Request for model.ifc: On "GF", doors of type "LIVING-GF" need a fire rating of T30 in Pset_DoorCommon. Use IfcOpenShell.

First a look at what the model holds.

```python
import ifcopenshell
import ifcopenshell.util.element

model = ifcopenshell.open("model.ifc")
print(model.schema)
storey = next(s for s in model.by_type("IfcBuildingStorey") if s.Name == "GF")
doors = [e for e in ifcopenshell.util.element.get_decomposition(storey) if e.is_a("IfcDoor")]
seen = {}
for e in doors:
    element_type = ifcopenshell.util.element.get_type(e)
    key = (element_type.Name if element_type != e and element_type else None, ifcopenshell.util.element.get_pset(e, "Pset_DoorCommon", "FireRating"))
    seen[key] = seen.get(key, 0) + 1
for (name, value), count in sorted(seen.items(), key=str):
    print(count, "x", name, "|", value)
```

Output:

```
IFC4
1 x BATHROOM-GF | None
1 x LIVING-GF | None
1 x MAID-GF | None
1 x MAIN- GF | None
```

```python
import ifcopenshell
import ifcopenshell.api.pset
import ifcopenshell.util.element

model = ifcopenshell.open("model.ifc")

storey = next(s for s in model.by_type("IfcBuildingStorey") if s.Name == "GF")
doors = [e for e in ifcopenshell.util.element.get_decomposition(storey) if e.is_a("IfcDoor")]

count = 0
for e in doors:
    element_type = ifcopenshell.util.element.get_type(e)
    if element_type in (None, e) or element_type.Name != "LIVING-GF":
        continue
    # add_pset returns the element's existing set when there is one.
    pset = ifcopenshell.api.pset.add_pset(model, product=e, name="Pset_DoorCommon")
    ifcopenshell.api.pset.edit_pset(model, pset=pset, properties={"FireRating": "T30"})
    count += 1

print(count, "doors updated")

model.write("model-out.ifc")
```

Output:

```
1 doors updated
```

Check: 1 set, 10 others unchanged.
